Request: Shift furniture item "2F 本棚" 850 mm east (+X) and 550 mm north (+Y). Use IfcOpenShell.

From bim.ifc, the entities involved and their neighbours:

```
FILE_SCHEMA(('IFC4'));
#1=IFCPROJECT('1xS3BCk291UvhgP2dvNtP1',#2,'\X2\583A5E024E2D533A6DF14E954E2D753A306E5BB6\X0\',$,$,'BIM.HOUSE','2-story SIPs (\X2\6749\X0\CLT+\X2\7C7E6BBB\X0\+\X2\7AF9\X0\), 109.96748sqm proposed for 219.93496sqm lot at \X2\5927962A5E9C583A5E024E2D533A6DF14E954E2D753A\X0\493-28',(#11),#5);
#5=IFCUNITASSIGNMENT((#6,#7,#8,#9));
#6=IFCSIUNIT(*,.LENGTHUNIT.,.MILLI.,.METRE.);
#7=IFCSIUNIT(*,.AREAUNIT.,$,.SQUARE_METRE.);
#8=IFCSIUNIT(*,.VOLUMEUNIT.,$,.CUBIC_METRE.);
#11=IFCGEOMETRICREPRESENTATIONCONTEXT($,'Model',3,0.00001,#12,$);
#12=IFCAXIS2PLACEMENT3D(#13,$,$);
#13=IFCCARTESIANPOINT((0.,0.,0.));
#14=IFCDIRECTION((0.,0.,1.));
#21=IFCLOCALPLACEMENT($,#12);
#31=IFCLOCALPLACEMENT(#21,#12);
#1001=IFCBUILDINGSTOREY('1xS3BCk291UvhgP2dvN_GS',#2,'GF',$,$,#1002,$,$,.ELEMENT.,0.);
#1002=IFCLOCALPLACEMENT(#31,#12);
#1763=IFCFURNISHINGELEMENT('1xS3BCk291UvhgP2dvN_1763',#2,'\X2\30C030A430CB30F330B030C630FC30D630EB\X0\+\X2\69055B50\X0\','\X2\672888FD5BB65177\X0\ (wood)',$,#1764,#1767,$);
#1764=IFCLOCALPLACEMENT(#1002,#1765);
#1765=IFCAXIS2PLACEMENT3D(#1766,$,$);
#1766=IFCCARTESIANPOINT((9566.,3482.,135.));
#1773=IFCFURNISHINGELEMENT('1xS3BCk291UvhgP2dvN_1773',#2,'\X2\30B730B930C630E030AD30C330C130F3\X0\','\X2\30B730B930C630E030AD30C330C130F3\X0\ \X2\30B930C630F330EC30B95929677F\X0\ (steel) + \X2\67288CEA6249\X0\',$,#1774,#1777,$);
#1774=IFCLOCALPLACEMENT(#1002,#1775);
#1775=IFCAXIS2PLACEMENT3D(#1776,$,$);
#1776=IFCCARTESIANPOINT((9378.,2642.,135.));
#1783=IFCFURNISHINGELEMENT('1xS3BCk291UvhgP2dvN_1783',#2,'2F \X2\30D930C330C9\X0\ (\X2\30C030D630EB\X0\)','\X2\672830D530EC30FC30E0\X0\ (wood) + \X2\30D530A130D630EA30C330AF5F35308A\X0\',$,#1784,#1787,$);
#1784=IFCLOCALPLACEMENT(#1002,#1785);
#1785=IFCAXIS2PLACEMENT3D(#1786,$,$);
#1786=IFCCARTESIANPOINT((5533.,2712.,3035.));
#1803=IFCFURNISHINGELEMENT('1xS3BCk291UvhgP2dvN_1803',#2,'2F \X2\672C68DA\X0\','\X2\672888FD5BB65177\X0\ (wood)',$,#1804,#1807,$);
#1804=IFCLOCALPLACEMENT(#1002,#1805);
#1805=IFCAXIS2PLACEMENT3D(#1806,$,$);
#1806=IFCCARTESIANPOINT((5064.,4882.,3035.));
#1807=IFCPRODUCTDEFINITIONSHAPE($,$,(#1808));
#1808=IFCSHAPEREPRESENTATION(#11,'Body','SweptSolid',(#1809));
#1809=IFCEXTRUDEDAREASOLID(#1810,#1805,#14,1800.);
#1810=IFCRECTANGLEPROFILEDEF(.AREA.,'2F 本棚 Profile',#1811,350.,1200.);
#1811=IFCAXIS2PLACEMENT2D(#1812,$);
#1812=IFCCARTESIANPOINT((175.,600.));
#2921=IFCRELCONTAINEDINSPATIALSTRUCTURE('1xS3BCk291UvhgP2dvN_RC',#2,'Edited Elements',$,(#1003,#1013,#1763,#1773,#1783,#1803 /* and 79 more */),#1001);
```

```python
import ifcopenshell
import ifcopenshell.api.geometry
import ifcopenshell.util.placement
import ifcopenshell.util.unit

model = ifcopenshell.open("bim.ifc")
unit_scale = ifcopenshell.util.unit.calculate_unit_scale(model)

item = model.by_guid("1xS3BCk291UvhgP2dvN_1803")
matrix = ifcopenshell.util.placement.get_local_placement(item.ObjectPlacement)
matrix[0, 3] += 0.85 / unit_scale
matrix[1, 3] += 0.55 / unit_scale
ifcopenshell.api.geometry.edit_object_placement(model, product=item, matrix=matrix, is_si=False)

print(ifcopenshell.util.placement.get_local_placement(item.ObjectPlacement).round(3) + 0.0)

model.write("bim_updated.ifc")
```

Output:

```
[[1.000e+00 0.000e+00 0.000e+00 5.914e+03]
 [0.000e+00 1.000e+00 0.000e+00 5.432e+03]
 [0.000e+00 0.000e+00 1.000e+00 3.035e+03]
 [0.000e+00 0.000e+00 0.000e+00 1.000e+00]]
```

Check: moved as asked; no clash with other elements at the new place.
